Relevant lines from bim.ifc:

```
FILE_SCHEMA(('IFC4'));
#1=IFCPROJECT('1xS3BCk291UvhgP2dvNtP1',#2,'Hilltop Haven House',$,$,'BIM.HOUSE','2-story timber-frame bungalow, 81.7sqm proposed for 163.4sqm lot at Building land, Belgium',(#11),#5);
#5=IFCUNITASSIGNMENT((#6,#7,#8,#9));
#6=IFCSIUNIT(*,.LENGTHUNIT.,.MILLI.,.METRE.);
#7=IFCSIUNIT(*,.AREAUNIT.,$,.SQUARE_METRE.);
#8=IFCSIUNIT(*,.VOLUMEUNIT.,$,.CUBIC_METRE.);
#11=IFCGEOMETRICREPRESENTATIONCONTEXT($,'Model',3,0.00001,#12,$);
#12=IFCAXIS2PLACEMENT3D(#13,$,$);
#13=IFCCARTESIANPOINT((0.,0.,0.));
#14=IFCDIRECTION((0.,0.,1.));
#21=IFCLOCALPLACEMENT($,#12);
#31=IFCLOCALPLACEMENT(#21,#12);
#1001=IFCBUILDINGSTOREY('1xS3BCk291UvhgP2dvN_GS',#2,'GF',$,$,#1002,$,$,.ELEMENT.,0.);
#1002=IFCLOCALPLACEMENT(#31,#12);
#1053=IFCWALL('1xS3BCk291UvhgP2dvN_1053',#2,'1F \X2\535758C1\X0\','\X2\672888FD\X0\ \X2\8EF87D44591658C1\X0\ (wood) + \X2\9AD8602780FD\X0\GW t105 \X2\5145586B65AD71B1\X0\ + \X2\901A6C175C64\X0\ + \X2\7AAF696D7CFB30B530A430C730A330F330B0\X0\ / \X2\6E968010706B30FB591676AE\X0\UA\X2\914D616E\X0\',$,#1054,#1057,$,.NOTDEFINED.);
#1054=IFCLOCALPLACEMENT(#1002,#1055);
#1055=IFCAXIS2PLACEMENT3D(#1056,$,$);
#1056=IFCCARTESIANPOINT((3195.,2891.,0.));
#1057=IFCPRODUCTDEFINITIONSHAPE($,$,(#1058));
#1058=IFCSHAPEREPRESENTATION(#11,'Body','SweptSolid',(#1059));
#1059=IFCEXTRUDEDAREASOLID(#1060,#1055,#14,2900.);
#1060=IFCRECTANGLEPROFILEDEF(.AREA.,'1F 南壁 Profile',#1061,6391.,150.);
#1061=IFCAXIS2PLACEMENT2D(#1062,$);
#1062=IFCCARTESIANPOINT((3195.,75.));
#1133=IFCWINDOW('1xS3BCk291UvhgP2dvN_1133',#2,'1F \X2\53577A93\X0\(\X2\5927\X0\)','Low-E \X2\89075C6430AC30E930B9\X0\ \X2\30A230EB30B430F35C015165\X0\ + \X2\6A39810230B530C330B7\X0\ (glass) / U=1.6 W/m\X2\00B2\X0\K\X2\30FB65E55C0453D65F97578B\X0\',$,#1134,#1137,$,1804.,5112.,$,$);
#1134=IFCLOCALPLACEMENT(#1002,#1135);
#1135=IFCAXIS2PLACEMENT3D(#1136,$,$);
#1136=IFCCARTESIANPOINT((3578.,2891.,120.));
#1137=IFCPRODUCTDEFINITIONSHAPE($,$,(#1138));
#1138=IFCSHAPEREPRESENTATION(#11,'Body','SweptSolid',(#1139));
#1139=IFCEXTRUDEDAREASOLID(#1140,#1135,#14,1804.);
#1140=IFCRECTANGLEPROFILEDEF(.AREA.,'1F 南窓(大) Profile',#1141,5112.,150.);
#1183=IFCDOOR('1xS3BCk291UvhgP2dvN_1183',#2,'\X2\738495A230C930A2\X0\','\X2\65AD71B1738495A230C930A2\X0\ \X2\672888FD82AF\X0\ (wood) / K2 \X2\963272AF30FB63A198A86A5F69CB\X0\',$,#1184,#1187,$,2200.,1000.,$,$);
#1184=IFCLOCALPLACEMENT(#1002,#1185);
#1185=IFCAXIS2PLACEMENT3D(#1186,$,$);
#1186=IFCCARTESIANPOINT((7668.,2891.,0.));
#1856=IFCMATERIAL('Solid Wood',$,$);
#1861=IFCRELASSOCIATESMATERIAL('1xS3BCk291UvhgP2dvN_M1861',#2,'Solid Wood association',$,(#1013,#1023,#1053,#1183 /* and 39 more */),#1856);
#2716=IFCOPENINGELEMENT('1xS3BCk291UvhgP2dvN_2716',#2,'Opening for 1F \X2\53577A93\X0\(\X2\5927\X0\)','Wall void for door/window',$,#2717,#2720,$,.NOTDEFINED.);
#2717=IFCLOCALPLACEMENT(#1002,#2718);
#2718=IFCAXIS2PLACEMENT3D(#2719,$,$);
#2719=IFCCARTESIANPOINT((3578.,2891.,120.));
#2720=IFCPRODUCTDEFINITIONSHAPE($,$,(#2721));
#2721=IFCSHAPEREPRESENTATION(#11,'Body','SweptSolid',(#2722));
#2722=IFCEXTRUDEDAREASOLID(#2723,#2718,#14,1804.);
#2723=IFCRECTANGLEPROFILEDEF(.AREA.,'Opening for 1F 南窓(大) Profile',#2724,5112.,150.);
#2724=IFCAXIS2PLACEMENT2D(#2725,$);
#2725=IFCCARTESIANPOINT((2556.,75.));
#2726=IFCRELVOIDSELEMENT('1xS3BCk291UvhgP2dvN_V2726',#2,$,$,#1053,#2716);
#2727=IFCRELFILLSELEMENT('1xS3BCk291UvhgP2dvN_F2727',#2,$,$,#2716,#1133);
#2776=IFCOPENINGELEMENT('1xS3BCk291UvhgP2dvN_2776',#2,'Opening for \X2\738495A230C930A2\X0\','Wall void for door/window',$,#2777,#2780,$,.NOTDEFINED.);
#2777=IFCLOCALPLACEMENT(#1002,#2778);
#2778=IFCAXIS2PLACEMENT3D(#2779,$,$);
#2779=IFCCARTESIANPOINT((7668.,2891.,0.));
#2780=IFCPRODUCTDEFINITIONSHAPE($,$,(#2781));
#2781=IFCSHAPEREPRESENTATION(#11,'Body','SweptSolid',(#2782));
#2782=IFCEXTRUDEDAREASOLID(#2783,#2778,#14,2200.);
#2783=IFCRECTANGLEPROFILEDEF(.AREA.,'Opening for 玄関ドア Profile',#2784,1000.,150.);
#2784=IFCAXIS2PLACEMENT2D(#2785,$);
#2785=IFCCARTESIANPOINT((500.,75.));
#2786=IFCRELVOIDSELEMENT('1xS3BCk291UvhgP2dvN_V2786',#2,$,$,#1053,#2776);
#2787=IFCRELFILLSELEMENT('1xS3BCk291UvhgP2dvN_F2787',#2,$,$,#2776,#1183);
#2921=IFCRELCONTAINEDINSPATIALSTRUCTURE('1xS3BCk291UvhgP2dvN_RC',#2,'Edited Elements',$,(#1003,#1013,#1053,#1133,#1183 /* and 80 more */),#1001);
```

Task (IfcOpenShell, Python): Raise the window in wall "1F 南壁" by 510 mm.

```python
import numpy as np
import ifcopenshell
import ifcopenshell.api.geometry
import ifcopenshell.util.placement
import ifcopenshell.util.unit

model = ifcopenshell.open("bim.ifc")
unit_scale = ifcopenshell.util.unit.calculate_unit_scale(model)

window = model.by_id(1133)
opening = window.FillsVoids[0].RelatingOpeningElement
dz = 510.0

shift = np.array([0.0, 0.0, dz])
# The window is not placed relative to its opening, so move both.
for product in (opening, window):
    matrix = ifcopenshell.util.placement.get_local_placement(product.ObjectPlacement)
    matrix[:3, 3] += shift
    ifcopenshell.api.geometry.edit_object_placement(model, product=product, matrix=matrix, is_si=False)

print(f"moved by {dz * unit_scale:+.3f} m")

model.write("bim_v2.ifc")
```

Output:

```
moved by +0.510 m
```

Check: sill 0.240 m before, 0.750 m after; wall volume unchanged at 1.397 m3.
